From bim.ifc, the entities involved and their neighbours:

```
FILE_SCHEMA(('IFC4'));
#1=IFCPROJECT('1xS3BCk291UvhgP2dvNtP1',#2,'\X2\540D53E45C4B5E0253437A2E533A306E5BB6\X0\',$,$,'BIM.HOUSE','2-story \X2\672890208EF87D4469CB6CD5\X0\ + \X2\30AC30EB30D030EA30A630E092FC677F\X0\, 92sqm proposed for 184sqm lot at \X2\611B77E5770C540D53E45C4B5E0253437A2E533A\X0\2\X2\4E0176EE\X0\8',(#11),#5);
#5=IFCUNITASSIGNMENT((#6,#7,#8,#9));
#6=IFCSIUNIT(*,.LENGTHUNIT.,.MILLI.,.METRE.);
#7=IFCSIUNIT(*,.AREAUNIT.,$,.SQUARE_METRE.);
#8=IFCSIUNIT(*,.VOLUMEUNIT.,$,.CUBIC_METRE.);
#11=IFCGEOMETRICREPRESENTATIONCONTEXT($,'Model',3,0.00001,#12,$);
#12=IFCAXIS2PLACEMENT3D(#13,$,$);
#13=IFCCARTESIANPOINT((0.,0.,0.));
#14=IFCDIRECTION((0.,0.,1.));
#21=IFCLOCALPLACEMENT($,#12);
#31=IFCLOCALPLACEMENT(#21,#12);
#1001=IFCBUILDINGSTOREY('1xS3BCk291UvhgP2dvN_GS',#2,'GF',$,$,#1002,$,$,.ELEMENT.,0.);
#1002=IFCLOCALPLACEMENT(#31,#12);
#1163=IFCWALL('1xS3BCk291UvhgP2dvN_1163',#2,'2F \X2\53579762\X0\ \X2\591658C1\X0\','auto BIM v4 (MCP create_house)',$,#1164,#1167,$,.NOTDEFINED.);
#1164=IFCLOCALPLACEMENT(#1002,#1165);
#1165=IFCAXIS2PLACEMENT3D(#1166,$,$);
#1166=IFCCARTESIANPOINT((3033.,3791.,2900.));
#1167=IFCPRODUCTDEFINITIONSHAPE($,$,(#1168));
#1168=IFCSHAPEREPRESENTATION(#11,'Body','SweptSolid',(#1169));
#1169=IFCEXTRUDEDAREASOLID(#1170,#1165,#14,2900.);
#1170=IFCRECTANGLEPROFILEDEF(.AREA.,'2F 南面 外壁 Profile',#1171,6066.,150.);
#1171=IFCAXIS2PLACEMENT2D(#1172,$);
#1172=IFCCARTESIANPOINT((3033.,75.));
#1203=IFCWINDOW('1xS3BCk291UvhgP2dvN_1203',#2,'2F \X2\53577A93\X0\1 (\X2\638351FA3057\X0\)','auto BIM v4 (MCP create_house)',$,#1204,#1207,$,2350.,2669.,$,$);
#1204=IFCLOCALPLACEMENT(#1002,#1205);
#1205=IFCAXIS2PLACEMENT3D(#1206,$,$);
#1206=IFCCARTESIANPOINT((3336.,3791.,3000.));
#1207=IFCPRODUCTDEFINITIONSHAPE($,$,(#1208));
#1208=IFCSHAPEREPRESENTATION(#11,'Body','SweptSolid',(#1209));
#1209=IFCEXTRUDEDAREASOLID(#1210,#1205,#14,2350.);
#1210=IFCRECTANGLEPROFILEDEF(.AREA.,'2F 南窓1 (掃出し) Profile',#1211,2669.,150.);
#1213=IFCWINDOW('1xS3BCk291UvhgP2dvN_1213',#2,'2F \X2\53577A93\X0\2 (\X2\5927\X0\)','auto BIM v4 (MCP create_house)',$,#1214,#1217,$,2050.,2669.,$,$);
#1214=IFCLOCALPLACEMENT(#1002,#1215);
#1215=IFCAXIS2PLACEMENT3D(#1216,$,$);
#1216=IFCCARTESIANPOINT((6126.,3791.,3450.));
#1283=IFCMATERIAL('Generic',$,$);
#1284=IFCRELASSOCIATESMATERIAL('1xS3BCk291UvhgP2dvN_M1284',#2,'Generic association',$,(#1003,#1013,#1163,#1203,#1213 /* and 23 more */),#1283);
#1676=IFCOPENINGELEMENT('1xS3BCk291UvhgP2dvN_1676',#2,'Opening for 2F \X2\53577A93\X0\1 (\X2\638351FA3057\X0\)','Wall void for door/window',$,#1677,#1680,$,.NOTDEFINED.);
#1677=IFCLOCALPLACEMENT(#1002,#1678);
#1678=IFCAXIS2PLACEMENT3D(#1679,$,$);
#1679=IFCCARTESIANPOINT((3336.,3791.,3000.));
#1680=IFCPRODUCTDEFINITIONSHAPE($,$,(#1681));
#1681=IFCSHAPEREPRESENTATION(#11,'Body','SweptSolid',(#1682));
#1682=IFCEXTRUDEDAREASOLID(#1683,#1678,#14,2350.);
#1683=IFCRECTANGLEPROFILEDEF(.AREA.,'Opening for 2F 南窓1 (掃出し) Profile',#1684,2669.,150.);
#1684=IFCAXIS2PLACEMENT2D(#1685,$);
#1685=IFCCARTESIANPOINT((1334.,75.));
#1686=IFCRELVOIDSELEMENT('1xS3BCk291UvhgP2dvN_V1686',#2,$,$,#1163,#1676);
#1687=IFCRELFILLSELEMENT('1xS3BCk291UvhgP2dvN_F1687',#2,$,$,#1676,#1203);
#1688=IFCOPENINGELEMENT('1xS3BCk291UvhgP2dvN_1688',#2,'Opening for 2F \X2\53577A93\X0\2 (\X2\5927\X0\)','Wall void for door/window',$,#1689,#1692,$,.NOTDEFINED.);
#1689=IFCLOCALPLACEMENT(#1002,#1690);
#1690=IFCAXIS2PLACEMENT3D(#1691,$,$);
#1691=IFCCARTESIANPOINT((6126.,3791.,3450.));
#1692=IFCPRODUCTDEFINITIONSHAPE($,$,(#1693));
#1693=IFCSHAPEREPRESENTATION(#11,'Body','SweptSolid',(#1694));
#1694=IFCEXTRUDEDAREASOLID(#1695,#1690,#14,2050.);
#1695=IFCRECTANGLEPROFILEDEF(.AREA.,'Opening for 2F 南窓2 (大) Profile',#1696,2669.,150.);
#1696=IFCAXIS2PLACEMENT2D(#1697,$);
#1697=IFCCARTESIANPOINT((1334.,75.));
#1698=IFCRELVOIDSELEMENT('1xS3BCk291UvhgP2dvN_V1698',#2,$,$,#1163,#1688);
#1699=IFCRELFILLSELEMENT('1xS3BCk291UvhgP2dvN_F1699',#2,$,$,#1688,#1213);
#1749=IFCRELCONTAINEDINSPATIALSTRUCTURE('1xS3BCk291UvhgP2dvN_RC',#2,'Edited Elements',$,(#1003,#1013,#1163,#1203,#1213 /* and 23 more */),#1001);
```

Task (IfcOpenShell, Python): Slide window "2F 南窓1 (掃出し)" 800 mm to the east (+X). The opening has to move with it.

```python
import ifcopenshell
import ifcopenshell.api.geometry
import ifcopenshell.util.placement
import ifcopenshell.util.unit

model = ifcopenshell.open("bim.ifc")
unit_scale = ifcopenshell.util.unit.calculate_unit_scale(model)

window = model.by_guid("1xS3BCk291UvhgP2dvN_1203")
opening = window.FillsVoids[0].RelatingOpeningElement
wall = opening.VoidsElements[0].RelatingBuildingElement

wall_matrix = ifcopenshell.util.placement.get_local_placement(wall.ObjectPlacement)
shift = wall_matrix[:3, 0] * 0.8 / unit_scale
before = ifcopenshell.util.placement.get_local_placement(window.ObjectPlacement)[:3, 3].copy()

# The window is not placed relative to its opening, so move both.
for product in (opening, window):
    matrix = ifcopenshell.util.placement.get_local_placement(product.ObjectPlacement)
    matrix[:3, 3] += shift
    ifcopenshell.api.geometry.edit_object_placement(model, product=product, matrix=matrix, is_si=False)

after = ifcopenshell.util.placement.get_local_placement(window.ObjectPlacement)[:3, 3]
print("window moved by", (after - before).round(3) + 0.0)

model.write("bim-out.ifc")
```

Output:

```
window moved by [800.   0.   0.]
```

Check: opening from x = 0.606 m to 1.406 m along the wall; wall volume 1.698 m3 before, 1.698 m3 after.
